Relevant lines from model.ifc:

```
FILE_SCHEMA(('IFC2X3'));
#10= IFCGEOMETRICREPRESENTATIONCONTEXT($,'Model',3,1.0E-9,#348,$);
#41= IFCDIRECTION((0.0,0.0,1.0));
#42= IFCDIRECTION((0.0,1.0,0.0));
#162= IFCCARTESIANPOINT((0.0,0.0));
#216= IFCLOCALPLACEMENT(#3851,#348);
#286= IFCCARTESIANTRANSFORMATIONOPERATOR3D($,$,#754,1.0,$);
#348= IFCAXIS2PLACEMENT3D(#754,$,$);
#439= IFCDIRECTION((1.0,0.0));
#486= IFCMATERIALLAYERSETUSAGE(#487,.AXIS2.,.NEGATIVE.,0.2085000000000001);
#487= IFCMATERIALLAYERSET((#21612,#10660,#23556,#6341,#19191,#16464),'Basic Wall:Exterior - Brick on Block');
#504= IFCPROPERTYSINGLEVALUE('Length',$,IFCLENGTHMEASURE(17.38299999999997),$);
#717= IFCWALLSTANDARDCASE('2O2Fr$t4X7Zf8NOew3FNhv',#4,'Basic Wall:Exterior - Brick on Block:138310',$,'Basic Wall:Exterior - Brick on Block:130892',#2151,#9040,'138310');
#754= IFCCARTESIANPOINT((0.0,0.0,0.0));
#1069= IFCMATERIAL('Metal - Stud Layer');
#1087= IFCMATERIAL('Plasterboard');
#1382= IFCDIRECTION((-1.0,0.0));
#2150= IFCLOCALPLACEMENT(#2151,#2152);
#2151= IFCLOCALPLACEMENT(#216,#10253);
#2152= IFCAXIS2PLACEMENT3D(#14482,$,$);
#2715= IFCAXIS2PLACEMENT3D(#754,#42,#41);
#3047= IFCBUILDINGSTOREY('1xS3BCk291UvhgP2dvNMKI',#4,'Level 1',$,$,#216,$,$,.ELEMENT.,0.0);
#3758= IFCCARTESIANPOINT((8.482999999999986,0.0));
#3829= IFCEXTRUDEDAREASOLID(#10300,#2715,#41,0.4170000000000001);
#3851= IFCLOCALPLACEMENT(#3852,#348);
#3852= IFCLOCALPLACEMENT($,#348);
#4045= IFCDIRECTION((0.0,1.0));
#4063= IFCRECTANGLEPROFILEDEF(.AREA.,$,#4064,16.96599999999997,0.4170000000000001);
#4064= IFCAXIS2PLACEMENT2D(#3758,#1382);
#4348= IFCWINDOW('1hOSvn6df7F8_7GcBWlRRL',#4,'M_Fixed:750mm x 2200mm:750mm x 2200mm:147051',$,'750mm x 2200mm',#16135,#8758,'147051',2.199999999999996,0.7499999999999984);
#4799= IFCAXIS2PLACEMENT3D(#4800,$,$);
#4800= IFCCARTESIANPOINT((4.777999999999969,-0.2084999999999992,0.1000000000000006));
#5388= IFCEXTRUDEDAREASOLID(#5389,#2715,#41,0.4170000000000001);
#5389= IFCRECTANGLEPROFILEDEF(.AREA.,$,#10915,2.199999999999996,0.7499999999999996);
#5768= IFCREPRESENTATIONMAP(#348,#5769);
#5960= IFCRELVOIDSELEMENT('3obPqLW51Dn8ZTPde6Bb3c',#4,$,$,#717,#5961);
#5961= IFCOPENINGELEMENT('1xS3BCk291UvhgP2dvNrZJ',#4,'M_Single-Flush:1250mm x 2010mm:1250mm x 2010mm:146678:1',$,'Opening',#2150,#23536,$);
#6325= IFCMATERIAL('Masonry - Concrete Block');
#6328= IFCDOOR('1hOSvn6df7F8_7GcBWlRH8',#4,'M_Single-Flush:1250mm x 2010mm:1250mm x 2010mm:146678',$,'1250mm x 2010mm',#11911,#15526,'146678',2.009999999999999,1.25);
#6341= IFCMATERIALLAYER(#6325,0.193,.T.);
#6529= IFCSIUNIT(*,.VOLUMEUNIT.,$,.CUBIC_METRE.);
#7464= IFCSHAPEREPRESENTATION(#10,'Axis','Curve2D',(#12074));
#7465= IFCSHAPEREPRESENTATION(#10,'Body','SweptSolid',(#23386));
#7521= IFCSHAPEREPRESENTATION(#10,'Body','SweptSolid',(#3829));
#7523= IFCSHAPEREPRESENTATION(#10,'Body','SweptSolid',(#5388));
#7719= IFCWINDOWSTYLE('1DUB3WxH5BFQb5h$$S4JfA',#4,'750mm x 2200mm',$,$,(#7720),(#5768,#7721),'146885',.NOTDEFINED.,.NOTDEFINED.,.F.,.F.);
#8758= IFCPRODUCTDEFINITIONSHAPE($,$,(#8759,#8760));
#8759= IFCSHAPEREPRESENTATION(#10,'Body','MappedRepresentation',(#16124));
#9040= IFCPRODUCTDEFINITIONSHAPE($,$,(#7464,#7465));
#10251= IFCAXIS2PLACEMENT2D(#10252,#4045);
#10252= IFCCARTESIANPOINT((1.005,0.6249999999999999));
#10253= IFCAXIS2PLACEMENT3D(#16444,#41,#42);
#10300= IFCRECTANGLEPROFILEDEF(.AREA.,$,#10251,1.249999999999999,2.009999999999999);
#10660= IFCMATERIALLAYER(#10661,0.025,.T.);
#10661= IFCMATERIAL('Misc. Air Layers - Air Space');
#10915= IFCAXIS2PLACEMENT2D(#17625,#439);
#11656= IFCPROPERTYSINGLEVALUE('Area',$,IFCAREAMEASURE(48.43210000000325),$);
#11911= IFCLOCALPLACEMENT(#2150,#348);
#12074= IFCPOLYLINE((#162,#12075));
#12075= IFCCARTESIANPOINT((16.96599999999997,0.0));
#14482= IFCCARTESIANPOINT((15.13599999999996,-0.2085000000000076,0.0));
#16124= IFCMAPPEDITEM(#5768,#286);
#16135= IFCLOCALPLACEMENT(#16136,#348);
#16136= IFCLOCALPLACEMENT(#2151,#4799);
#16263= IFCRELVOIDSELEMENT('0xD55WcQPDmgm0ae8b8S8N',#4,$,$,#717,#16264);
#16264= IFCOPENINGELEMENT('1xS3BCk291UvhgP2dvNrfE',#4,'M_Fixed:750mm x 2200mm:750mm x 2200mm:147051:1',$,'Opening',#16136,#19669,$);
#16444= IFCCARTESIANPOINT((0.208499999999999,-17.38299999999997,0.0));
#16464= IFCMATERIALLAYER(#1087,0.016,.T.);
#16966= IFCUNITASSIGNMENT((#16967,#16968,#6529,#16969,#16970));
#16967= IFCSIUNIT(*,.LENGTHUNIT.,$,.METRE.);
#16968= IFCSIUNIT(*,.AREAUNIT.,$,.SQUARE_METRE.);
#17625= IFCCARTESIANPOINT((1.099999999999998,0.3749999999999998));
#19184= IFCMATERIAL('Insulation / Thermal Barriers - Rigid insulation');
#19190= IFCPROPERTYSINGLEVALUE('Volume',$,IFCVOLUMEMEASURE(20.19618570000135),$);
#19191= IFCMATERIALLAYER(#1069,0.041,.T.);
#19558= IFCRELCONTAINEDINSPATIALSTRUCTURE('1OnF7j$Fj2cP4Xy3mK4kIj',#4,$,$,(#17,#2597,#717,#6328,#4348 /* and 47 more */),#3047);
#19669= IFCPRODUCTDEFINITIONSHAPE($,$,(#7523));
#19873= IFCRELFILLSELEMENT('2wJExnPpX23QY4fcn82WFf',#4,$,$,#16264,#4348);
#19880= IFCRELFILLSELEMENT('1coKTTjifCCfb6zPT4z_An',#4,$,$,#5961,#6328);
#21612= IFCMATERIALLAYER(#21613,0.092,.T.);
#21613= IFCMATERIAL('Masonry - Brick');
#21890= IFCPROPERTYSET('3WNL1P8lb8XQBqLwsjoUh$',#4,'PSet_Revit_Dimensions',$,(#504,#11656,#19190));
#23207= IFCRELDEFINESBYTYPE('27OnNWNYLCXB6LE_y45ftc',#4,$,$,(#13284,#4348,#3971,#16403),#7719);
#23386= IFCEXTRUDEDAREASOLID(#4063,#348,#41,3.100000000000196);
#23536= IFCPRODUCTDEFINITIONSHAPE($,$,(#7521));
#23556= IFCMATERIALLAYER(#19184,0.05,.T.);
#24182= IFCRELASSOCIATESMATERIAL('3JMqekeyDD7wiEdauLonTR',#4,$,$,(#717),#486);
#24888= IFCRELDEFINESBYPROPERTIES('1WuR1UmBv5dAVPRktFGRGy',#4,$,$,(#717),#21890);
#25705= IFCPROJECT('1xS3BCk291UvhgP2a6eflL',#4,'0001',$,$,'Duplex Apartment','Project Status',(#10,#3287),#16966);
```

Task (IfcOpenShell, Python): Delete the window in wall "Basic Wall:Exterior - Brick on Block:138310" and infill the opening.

```python
import ifcopenshell
import ifcopenshell.api.feature
import ifcopenshell.api.pset
import ifcopenshell.api.root
import ifcopenshell.geom
import ifcopenshell.util.element
import ifcopenshell.util.shape
import ifcopenshell.util.unit

model = ifcopenshell.open("model.ifc")
area_scale = ifcopenshell.util.unit.calculate_unit_scale(model, "AREAUNIT")
volume_scale = ifcopenshell.util.unit.calculate_unit_scale(model, "VOLUMEUNIT")
settings = ifcopenshell.geom.settings()


def volume(element):
    """Net volume in cubic metres, openings subtracted."""
    shape = ifcopenshell.geom.create_shape(settings, element)
    return ifcopenshell.util.shape.get_volume(shape.geometry)


window = model.by_id(4348)
opening = window.FillsVoids[0].RelatingOpeningElement
wall = opening.VoidsElements[0].RelatingBuildingElement
before = volume(wall)

ifcopenshell.api.root.remove_product(model, product=window)
ifcopenshell.api.feature.remove_feature(model, feature=opening)

after = volume(wall)
thickness = 0.417  # wall thickness in metres

# Update the wall's stored quantities.
pset = model.by_id(ifcopenshell.util.element.get_pset(wall, "PSet_Revit_Dimensions", should_inherit=False)["id"])
ifcopenshell.api.pset.edit_pset(model, pset=pset, properties={
    "Area": model.create_entity("IfcAreaMeasure", after / thickness / area_scale),
    "Volume": model.create_entity("IfcVolumeMeasure", after / volume_scale),
})

print(f"wall volume {before:.3f} -> {after:.3f} m3")

model.write("model_v2.ifc")
```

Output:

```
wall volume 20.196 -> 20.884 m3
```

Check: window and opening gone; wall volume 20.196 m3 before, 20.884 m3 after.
